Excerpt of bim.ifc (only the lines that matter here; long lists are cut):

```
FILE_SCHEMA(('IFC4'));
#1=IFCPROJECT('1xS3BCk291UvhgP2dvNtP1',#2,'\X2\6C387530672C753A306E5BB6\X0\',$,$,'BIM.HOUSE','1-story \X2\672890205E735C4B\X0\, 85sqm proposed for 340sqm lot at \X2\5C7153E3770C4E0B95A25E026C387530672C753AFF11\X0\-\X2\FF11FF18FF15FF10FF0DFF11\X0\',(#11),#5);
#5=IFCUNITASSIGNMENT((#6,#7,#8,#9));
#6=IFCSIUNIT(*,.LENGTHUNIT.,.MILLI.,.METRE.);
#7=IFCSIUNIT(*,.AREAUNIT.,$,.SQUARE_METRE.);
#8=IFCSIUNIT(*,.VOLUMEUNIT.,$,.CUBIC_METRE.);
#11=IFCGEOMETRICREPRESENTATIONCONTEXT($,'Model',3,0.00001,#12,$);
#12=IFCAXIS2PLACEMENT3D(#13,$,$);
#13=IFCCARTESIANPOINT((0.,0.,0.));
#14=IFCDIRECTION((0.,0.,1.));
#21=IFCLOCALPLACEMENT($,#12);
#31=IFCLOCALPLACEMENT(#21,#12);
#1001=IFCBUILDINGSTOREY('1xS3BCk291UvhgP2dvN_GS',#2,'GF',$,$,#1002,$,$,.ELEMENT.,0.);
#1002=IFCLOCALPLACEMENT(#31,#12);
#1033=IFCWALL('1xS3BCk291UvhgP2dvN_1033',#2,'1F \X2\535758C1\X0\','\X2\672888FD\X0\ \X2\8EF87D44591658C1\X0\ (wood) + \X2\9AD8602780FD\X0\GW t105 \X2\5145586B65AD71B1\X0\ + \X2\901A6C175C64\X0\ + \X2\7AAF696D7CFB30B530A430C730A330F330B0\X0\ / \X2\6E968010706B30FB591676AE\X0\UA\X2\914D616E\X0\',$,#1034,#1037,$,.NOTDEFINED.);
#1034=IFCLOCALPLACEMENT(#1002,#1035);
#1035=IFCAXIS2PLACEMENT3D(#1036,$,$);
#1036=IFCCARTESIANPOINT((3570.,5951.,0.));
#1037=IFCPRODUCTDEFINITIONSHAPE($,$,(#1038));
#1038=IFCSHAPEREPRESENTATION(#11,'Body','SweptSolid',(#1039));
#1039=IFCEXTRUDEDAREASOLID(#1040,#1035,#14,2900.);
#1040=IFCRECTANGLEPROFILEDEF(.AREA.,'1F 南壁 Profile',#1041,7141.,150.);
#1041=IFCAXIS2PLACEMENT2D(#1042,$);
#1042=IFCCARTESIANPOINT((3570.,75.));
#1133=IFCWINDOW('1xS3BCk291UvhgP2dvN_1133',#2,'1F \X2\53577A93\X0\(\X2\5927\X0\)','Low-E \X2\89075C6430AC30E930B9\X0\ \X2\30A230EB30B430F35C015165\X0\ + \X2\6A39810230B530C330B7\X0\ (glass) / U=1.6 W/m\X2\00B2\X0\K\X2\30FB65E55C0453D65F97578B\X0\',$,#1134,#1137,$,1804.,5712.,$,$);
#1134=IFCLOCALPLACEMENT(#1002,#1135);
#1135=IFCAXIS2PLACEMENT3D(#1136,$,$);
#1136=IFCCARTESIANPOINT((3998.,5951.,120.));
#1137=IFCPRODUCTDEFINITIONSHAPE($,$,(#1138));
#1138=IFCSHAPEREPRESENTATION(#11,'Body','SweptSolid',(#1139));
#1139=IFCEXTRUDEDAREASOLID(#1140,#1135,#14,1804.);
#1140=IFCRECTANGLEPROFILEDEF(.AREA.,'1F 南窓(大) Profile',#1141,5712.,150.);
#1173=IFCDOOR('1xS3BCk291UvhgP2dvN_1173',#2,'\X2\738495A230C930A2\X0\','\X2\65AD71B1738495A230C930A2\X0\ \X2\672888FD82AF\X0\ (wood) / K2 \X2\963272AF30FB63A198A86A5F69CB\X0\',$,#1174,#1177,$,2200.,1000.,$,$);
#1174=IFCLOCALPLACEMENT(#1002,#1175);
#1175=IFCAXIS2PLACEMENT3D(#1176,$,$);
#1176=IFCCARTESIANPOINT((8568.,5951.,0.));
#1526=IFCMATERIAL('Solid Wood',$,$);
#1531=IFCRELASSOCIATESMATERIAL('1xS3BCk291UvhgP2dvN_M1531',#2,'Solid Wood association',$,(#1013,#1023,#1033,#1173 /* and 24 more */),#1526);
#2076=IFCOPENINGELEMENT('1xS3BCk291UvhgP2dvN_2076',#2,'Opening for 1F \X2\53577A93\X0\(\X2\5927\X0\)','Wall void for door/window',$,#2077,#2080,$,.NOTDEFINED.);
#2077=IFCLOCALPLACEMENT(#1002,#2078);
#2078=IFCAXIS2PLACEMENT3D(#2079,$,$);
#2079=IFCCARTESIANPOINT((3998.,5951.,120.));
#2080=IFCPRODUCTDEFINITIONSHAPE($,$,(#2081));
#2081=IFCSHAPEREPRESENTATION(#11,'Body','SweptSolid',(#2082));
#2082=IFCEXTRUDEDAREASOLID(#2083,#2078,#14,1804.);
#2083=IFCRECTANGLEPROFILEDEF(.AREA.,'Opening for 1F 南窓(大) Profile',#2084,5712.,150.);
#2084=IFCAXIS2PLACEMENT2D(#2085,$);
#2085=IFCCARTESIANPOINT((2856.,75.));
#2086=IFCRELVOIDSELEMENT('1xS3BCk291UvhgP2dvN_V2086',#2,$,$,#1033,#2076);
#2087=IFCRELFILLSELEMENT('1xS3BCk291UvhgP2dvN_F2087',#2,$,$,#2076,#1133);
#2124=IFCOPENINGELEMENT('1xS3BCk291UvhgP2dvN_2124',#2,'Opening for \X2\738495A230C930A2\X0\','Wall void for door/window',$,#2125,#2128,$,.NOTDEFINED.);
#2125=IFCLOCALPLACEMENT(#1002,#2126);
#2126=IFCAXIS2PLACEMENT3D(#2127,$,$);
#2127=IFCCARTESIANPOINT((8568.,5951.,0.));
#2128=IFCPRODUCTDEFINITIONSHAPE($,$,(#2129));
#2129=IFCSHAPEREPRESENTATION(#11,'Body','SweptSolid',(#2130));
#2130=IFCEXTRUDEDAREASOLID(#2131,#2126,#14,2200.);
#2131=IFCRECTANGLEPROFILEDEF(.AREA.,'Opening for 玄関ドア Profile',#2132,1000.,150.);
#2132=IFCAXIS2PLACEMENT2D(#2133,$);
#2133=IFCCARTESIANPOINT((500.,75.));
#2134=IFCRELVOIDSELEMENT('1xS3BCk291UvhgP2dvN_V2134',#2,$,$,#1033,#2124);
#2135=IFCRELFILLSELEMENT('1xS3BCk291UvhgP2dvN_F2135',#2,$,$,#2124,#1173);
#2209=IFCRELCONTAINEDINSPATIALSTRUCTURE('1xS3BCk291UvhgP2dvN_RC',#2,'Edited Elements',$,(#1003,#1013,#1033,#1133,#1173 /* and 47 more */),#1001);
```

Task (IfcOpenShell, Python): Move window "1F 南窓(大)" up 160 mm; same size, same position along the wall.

```python
import numpy as np
import ifcopenshell
import ifcopenshell.api.geometry
import ifcopenshell.util.placement
import ifcopenshell.util.unit

model = ifcopenshell.open("bim.ifc")
unit_scale = ifcopenshell.util.unit.calculate_unit_scale(model)

window = model.by_id(1133)
opening = window.FillsVoids[0].RelatingOpeningElement
dz = 0.16 / unit_scale

shift = np.array([0.0, 0.0, dz])
# The window is not placed relative to its opening, so move both.
for product in (opening, window):
    matrix = ifcopenshell.util.placement.get_local_placement(product.ObjectPlacement)
    matrix[:3, 3] += shift
    ifcopenshell.api.geometry.edit_object_placement(model, product=product, matrix=matrix, is_si=False)

print(f"moved by {dz * unit_scale:+.3f} m")

model.write("bim_rev.ifc")
```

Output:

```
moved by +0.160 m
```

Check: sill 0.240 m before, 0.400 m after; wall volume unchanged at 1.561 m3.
